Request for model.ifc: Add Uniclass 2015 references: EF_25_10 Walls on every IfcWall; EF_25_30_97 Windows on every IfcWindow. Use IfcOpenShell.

First a look at what the model holds.

```python
import ifcopenshell

model = ifcopenshell.open("model.ifc")
print(model.schema)
print("classifications:", [c.Name for c in model.by_type("IfcClassification")])
for ifc_class in ("IfcDoor", "IfcRoof", "IfcStair", "IfcWall", "IfcWindow"):
    print(ifc_class, len(model.by_type(ifc_class)))
```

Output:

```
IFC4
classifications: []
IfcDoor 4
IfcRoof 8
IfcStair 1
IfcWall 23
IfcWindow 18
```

```python
import ifcopenshell
import ifcopenshell.api.classification

model = ifcopenshell.open("model.ifc")

system = ifcopenshell.api.classification.add_classification(model, classification="Uniclass 2015")

codes = {
    "IfcWall": ("EF_25_10", "Walls"),
    "IfcWindow": ("EF_25_30_97", "Windows"),
}
for ifc_class, (code, name) in codes.items():
    products = model.by_type(ifc_class)
    ifcopenshell.api.classification.add_reference(
        model, products=products, classification=system, identification=code, name=name
    )
    print(code, len(products))

model.write("model_updated.ifc")
```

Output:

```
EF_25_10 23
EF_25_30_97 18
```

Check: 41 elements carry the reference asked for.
